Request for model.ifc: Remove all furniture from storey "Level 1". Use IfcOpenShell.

First a look at what the model holds.

```python
import ifcopenshell
import ifcopenshell.util.element

model = ifcopenshell.open("model.ifc")
print(model.schema)
storey = next(s for s in model.by_type("IfcBuildingStorey") if s.Name == "Level 1")
furniture = [e for e in ifcopenshell.util.element.get_decomposition(storey) if e.is_a("IfcFurnishingElement")]
seen = {}
for e in furniture:
    element_type = ifcopenshell.util.element.get_type(e)
    name = element_type.Name if element_type not in (None, e) else None
    seen[name] = seen.get(name, 0) + 1
for name, count in sorted(seen.items(), key=str):
    print(count, "x", name)
```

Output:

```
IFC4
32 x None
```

```python
import ifcopenshell
import ifcopenshell.api.root
import ifcopenshell.util.element

model = ifcopenshell.open("model.ifc")

storey = next(s for s in model.by_type("IfcBuildingStorey") if s.Name == "Level 1")
furniture = [e for e in ifcopenshell.util.element.get_decomposition(storey) if e.is_a("IfcFurnishingElement")]

for e in furniture:
    ifcopenshell.api.root.remove_product(model, product=e)
print(len(furniture), "removed")

model.write("model_edited.ifc")
```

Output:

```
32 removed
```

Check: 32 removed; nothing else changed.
